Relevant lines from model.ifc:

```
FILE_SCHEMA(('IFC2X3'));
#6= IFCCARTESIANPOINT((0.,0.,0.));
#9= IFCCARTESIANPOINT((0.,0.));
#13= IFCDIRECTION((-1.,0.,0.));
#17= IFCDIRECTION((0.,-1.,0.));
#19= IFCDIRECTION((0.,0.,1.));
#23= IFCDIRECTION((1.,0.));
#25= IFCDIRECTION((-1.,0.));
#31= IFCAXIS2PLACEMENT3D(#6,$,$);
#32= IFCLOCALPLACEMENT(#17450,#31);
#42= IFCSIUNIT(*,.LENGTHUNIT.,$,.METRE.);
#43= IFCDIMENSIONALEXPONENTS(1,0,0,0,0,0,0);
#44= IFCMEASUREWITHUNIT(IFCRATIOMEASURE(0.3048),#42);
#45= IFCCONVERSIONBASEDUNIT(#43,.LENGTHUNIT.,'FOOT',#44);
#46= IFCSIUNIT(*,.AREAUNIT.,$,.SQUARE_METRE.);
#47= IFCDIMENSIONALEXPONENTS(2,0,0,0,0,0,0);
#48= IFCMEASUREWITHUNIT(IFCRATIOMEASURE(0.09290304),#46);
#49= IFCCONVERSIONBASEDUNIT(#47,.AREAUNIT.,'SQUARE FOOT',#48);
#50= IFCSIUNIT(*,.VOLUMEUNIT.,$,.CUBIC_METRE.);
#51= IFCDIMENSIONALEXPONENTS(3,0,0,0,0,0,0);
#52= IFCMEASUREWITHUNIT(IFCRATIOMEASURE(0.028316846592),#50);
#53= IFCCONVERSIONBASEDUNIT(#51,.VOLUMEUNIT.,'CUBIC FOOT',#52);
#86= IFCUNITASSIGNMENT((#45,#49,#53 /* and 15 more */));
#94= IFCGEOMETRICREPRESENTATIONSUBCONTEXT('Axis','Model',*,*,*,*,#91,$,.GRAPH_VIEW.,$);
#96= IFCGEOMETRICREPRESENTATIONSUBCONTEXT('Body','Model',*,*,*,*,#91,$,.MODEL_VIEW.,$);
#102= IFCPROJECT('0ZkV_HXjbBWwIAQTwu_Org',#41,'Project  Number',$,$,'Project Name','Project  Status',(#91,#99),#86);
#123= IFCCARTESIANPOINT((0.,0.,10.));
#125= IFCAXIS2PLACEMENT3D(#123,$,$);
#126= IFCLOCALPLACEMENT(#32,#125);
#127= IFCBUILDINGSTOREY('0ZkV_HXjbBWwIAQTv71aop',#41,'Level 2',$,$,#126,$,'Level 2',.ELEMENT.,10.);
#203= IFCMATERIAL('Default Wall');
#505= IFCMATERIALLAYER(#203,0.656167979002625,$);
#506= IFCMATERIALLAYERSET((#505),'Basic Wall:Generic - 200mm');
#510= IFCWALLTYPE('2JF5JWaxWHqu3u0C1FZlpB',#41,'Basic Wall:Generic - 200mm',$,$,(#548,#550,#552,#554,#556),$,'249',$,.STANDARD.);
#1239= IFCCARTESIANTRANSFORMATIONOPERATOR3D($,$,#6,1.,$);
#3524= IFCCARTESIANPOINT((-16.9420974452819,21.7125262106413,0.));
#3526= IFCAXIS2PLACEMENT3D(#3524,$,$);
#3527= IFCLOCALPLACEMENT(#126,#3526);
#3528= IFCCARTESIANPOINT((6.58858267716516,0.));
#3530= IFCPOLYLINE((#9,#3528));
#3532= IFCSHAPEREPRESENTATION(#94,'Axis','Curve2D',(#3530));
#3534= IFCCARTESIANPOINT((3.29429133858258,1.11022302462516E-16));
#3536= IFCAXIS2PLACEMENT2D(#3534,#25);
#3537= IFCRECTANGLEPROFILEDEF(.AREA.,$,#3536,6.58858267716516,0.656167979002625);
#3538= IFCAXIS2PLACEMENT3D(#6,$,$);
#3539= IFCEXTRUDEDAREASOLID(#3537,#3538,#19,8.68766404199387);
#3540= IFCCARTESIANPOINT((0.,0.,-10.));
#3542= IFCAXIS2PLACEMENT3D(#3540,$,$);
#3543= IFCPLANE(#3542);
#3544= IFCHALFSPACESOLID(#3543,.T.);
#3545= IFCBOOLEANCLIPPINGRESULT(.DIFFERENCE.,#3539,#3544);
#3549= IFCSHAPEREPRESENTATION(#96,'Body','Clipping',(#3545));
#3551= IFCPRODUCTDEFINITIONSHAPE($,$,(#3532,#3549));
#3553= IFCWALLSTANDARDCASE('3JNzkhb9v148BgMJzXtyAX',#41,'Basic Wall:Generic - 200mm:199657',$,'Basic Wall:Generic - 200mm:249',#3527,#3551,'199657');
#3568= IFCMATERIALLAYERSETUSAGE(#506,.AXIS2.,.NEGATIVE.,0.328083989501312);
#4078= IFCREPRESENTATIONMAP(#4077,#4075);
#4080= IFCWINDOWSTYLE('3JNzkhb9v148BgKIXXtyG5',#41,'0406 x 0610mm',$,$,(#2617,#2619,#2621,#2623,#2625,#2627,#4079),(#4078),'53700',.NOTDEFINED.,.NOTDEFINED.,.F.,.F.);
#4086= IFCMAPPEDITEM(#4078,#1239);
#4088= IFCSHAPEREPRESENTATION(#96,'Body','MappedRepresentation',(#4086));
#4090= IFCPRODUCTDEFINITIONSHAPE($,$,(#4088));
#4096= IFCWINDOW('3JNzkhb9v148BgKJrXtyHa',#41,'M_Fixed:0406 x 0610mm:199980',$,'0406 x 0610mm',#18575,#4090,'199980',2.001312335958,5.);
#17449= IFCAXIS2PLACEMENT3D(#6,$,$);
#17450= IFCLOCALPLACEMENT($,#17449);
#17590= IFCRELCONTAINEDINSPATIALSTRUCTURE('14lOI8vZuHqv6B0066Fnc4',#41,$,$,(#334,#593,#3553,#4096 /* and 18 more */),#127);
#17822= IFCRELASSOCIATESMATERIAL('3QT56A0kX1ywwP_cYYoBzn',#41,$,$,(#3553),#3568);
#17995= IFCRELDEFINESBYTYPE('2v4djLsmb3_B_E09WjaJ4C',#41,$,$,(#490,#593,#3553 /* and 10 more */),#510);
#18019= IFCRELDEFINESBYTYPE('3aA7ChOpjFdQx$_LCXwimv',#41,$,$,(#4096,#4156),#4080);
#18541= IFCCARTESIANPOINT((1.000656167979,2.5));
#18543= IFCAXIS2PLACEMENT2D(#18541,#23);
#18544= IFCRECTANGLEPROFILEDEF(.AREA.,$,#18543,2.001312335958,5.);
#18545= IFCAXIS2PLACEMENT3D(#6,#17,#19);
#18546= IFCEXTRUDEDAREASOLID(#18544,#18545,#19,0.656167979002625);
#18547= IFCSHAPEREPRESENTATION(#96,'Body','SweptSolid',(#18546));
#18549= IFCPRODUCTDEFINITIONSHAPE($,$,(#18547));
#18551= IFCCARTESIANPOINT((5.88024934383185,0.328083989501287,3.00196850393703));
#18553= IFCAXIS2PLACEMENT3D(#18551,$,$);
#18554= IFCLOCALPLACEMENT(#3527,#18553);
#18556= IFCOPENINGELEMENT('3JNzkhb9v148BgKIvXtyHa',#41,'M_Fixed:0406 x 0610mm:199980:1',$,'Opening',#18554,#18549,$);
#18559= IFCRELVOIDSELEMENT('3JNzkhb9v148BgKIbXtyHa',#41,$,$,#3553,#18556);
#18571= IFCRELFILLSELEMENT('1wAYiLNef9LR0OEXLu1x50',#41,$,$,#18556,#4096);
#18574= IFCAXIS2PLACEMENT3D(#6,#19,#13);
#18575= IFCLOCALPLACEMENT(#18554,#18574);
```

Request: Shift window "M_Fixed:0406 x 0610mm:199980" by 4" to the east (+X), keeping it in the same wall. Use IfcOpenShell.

```python
import ifcopenshell
import ifcopenshell.api.geometry
import ifcopenshell.util.placement
import ifcopenshell.util.unit

model = ifcopenshell.open("model.ifc")
unit_scale = ifcopenshell.util.unit.calculate_unit_scale(model)

window = model.by_guid("3JNzkhb9v148BgKJrXtyHa")
opening = window.FillsVoids[0].RelatingOpeningElement
wall = opening.VoidsElements[0].RelatingBuildingElement

wall_matrix = ifcopenshell.util.placement.get_local_placement(wall.ObjectPlacement)
shift = wall_matrix[:3, 0] * 4 * 0.0254 / unit_scale
before = ifcopenshell.util.placement.get_local_placement(window.ObjectPlacement)[:3, 3].copy()

# The window is placed relative to its opening, so it follows when the opening moves.
matrix = ifcopenshell.util.placement.get_local_placement(opening.ObjectPlacement)
matrix[:3, 3] += shift
ifcopenshell.api.geometry.edit_object_placement(
    model, product=opening, matrix=matrix, is_si=False, should_transform_children=True
)

after = ifcopenshell.util.placement.get_local_placement(window.ObjectPlacement)[:3, 3]
print("window moved by", (after - before).round(3) + 0.0)

model.write("model_rev.ifc")
```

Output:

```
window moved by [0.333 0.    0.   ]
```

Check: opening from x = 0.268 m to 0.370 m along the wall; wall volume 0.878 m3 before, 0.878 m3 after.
